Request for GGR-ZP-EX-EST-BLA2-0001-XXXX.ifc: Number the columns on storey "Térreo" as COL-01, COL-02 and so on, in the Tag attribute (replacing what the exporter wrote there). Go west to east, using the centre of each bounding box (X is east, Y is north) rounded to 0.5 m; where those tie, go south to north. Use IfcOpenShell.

First a look at what the model holds.

```python
import ifcopenshell
import ifcopenshell.util.element
import ifcopenshell.util.placement

model = ifcopenshell.open("GGR-ZP-EX-EST-BLA2-0001-XXXX.ifc")
print(model.schema)
storey = next(s for s in model.by_type("IfcBuildingStorey") if s.Name == "Térreo")
columns = [e for e in ifcopenshell.util.element.get_decomposition(storey) if e.is_a("IfcColumn")]
for e in sorted(columns, key=lambda e: e.id()):
    origin = ifcopenshell.util.placement.get_local_placement(e.ObjectPlacement)[:3, 3]
    print(e.id(), e.Tag, e.Name, origin.round(2) + 0.0, sep=" | ")
```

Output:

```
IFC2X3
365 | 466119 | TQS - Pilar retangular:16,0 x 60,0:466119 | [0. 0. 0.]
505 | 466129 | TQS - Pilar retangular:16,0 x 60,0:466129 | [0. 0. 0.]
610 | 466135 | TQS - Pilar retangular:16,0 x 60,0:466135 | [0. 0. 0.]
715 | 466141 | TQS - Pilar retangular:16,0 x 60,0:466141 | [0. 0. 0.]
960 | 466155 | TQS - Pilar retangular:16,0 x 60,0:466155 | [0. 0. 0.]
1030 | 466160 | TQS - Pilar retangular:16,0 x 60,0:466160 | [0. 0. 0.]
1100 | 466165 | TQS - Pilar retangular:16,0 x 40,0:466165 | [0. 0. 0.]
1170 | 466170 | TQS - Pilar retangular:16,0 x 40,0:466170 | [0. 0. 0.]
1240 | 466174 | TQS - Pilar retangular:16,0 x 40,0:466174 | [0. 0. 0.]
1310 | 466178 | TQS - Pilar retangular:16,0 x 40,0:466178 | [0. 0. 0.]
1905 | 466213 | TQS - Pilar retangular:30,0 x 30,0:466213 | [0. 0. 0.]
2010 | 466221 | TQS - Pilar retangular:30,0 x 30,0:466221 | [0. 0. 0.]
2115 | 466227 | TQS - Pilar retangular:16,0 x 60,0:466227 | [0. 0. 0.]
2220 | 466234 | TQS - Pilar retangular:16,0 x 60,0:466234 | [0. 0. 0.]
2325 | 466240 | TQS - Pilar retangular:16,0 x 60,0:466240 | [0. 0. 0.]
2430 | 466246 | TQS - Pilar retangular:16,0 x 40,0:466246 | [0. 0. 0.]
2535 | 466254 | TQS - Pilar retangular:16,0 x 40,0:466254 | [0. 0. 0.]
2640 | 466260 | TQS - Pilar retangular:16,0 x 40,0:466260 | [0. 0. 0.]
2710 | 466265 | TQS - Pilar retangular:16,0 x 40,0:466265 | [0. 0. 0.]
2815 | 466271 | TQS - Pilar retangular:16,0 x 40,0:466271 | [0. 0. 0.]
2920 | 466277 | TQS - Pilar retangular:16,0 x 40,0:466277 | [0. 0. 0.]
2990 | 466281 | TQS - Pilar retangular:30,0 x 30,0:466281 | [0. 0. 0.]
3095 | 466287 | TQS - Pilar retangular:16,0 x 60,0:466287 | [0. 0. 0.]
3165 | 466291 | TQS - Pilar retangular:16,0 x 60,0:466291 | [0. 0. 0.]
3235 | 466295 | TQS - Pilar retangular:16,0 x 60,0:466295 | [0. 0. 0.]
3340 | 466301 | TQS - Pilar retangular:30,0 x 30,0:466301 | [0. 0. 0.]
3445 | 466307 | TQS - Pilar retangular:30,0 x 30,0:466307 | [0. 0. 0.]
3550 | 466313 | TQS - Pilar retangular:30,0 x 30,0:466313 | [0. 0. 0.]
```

```python
import ifcopenshell
import ifcopenshell.geom
import ifcopenshell.util.element
import ifcopenshell.util.shape

model = ifcopenshell.open("GGR-ZP-EX-EST-BLA2-0001-XXXX.ifc")
settings = ifcopenshell.geom.settings()
settings.set("use-world-coords", True)


def centre(element):
    shape = ifcopenshell.geom.create_shape(settings, element)
    return ifcopenshell.util.shape.get_bbox_centroid(shape.geometry)


storey = next(s for s in model.by_type("IfcBuildingStorey") if s.Name == "Térreo")
columns = [e for e in ifcopenshell.util.element.get_decomposition(storey) if e.is_a("IfcColumn")]

# Insertion points can sit at a corner or the storey origin, so sort by the geometry (in metres).
centres = {e: centre(e) for e in columns}
columns.sort(key=lambda e: (round(centres[e][0] / 0.5), centres[e][1]))

for i, e in enumerate(columns, start=1):
    number = f"COL-{i:02d}"
    e.Tag = number
    print(e.id(), number)

model.write("GGR-ZP-EX-EST-BLA2-0001-XXXX-out.ifc")
```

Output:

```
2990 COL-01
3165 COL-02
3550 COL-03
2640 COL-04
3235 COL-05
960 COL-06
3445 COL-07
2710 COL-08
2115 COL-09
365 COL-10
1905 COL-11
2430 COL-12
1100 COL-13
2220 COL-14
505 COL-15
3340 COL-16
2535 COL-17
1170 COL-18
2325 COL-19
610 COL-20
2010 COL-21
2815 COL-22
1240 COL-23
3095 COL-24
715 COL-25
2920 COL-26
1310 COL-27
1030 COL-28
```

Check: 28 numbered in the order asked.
